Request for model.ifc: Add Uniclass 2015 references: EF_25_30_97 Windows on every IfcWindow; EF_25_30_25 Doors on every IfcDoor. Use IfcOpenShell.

First a look at what the model holds.

```python
import ifcopenshell

model = ifcopenshell.open("model.ifc")
print(model.schema)
print("classifications:", [c.Name for c in model.by_type("IfcClassification")])
for ifc_class in ("IfcDoor", "IfcRoof", "IfcStair", "IfcWall", "IfcWindow"):
    print(ifc_class, len(model.by_type(ifc_class)))
```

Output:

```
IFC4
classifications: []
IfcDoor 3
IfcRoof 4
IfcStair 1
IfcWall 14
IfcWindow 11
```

```python
import ifcopenshell
import ifcopenshell.api.classification

model = ifcopenshell.open("model.ifc")

system = ifcopenshell.api.classification.add_classification(model, classification="Uniclass 2015")

codes = {
    "IfcWindow": ("EF_25_30_97", "Windows"),
    "IfcDoor": ("EF_25_30_25", "Doors"),
}
for ifc_class, (code, name) in codes.items():
    products = model.by_type(ifc_class)
    ifcopenshell.api.classification.add_reference(
        model, products=products, classification=system, identification=code, name=name
    )
    print(code, len(products))

model.write("model_edited.ifc")
```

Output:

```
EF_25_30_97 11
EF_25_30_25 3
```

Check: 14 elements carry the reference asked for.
